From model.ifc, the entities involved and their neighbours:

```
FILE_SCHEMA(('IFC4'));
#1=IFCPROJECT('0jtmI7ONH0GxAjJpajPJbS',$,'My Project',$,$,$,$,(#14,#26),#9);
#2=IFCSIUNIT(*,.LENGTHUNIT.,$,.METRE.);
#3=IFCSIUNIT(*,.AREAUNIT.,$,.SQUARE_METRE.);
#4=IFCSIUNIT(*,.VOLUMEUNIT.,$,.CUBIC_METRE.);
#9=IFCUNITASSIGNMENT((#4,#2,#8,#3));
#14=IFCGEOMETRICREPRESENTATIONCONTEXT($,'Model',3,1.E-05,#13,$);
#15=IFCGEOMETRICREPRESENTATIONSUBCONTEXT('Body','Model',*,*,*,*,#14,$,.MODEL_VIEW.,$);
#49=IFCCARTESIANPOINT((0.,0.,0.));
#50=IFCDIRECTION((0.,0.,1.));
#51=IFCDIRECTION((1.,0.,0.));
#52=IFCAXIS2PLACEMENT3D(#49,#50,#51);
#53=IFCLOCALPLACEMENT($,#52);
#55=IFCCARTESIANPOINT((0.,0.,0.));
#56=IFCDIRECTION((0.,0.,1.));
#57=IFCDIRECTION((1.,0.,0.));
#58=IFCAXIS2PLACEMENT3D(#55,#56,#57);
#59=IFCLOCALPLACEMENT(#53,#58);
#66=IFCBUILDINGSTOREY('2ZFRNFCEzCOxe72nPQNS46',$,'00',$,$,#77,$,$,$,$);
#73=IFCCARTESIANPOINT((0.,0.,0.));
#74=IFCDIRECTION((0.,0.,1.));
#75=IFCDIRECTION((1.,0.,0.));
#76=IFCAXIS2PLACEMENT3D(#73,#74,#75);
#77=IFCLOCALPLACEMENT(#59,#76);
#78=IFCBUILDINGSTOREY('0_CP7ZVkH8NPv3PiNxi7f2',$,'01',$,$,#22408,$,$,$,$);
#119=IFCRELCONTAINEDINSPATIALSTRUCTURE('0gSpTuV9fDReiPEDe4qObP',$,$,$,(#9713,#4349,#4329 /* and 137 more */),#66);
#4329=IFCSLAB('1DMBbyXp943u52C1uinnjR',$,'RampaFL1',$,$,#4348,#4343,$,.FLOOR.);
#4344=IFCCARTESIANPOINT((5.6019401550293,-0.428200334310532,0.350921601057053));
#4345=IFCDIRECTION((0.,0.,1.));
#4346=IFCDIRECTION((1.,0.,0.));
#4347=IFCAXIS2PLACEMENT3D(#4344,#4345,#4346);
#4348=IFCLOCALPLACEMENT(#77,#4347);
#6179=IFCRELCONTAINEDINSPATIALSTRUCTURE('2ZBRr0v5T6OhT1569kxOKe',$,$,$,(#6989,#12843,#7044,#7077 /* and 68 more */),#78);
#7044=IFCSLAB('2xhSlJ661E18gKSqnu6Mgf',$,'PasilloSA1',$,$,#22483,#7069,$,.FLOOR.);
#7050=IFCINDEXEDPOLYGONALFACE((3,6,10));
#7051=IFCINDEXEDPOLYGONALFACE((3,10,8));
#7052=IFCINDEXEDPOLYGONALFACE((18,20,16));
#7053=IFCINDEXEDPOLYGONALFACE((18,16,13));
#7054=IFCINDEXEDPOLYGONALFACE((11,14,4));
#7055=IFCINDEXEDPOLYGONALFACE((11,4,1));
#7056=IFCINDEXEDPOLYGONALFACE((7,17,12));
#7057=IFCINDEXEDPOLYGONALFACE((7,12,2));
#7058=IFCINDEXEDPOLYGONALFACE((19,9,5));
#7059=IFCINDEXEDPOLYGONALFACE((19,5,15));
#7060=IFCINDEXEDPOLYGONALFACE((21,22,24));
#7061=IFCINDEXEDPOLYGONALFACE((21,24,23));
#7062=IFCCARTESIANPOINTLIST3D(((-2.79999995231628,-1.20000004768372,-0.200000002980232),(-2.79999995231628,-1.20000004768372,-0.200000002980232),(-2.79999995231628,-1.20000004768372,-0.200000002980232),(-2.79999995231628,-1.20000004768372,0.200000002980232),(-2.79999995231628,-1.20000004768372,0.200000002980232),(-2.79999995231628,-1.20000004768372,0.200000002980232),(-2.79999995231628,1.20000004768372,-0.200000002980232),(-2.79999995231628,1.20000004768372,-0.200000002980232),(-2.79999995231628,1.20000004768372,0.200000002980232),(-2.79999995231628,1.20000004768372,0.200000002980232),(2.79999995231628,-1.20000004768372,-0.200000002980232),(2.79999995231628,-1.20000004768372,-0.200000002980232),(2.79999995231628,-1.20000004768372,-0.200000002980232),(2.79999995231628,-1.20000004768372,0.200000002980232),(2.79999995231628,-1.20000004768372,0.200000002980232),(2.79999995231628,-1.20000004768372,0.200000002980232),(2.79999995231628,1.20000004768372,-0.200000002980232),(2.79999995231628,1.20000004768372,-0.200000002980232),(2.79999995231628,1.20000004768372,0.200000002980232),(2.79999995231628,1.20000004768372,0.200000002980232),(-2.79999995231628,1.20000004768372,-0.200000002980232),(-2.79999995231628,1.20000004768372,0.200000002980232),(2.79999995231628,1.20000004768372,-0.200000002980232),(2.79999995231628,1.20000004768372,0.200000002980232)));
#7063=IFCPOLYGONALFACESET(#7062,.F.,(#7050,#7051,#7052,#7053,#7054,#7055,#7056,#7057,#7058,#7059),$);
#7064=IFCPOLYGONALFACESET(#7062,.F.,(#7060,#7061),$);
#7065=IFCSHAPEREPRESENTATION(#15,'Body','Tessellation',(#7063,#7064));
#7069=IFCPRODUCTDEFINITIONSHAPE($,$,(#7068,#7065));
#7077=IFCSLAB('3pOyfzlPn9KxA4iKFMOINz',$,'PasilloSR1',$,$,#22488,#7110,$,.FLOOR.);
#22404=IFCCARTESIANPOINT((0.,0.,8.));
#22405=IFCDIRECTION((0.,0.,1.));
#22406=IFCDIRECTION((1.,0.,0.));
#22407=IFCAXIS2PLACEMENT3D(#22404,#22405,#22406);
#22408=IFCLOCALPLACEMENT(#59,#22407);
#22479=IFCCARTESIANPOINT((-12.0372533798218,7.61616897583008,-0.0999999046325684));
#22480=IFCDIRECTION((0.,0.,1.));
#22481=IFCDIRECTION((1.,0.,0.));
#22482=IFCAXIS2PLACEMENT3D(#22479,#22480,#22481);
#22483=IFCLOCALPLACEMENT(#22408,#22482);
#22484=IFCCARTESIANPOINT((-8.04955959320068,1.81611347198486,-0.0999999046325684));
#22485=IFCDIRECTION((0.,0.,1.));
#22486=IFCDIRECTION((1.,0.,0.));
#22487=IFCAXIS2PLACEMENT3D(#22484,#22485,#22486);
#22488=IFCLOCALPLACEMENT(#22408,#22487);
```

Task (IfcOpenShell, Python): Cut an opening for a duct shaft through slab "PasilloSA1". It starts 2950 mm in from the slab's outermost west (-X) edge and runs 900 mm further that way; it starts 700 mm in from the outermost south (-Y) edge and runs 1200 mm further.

```python
import numpy as np
import ifcopenshell
import ifcopenshell.api.feature
import ifcopenshell.api.geometry
import ifcopenshell.api.root
import ifcopenshell.geom
import ifcopenshell.util.placement
import ifcopenshell.util.representation
import ifcopenshell.util.shape
import ifcopenshell.util.unit

model = ifcopenshell.open("model.ifc")
unit_scale = ifcopenshell.util.unit.calculate_unit_scale(model)
settings = ifcopenshell.geom.settings()


def volume(element):
    """Net volume in cubic metres, openings subtracted."""
    shape = ifcopenshell.geom.create_shape(settings, element)
    return ifcopenshell.util.shape.get_volume(shape.geometry)


slab = model.by_guid("2xhSlJ661E18gKSqnu6Mgf")
before = volume(slab)

# Extent in the slab's own axes, in metres. The edges named are its -X and -Y sides.
slab_shape = ifcopenshell.geom.create_shape(settings, slab)
vertices = ifcopenshell.util.shape.get_vertices(slab_shape.geometry)
x_min, y_min, bottom = vertices.min(axis=0)
top = vertices[:, 2].max()

opening = ifcopenshell.api.root.create_entity(model, ifc_class="IfcOpeningElement", name="Duct shaft opening", predefined_type="OPENING")
context = ifcopenshell.util.representation.get_context(model, "Model", "Body", "MODEL_VIEW")
width, depth = 0.9, 1.2
outline = [(0.0, 0.0), (width, 0.0), (width, depth), (0.0, depth), (0.0, 0.0)]
# Overshoot both faces by 50 mm so the cut is clean.
shape = ifcopenshell.api.geometry.add_slab_representation(
    model, context=context, depth=top - bottom + 0.1, polyline=outline
)
ifcopenshell.api.geometry.assign_representation(model, product=opening, representation=shape)

matrix = ifcopenshell.util.placement.get_local_placement(slab.ObjectPlacement)
matrix[:, 3] = matrix @ np.append(np.array([x_min + 2.95, y_min + 0.7, bottom - 0.05]) / unit_scale, 1.0)
ifcopenshell.api.geometry.edit_object_placement(model, product=opening, matrix=matrix, is_si=False)
ifcopenshell.api.feature.add_feature(model, feature=opening, element=slab)

after = volume(slab)

print(f"slab volume {before:.3f} -> {after:.3f} m3")

model.write("model_v2.ifc")
```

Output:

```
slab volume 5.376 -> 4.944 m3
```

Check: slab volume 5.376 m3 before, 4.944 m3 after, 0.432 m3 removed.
